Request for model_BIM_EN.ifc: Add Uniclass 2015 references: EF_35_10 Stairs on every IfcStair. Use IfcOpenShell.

First a look at what the model holds.

```python
import ifcopenshell

model = ifcopenshell.open("model_BIM_EN.ifc")
print(model.schema)
print("classifications:", [c.Name for c in model.by_type("IfcClassification")])
for ifc_class in ("IfcDoor", "IfcRoof", "IfcStair", "IfcWall", "IfcWindow"):
    print(ifc_class, len(model.by_type(ifc_class)))
```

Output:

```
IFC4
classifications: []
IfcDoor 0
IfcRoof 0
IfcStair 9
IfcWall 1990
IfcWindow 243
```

```python
import ifcopenshell
import ifcopenshell.api.classification

model = ifcopenshell.open("model_BIM_EN.ifc")

system = ifcopenshell.api.classification.add_classification(model, classification="Uniclass 2015")

codes = {
    "IfcStair": ("EF_35_10", "Stairs"),
}
for ifc_class, (code, name) in codes.items():
    products = model.by_type(ifc_class)
    ifcopenshell.api.classification.add_reference(
        model, products=products, classification=system, identification=code, name=name
    )
    print(code, len(products))

model.write("model_BIM_EN_v2.ifc")
```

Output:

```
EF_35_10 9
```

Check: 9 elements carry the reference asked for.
